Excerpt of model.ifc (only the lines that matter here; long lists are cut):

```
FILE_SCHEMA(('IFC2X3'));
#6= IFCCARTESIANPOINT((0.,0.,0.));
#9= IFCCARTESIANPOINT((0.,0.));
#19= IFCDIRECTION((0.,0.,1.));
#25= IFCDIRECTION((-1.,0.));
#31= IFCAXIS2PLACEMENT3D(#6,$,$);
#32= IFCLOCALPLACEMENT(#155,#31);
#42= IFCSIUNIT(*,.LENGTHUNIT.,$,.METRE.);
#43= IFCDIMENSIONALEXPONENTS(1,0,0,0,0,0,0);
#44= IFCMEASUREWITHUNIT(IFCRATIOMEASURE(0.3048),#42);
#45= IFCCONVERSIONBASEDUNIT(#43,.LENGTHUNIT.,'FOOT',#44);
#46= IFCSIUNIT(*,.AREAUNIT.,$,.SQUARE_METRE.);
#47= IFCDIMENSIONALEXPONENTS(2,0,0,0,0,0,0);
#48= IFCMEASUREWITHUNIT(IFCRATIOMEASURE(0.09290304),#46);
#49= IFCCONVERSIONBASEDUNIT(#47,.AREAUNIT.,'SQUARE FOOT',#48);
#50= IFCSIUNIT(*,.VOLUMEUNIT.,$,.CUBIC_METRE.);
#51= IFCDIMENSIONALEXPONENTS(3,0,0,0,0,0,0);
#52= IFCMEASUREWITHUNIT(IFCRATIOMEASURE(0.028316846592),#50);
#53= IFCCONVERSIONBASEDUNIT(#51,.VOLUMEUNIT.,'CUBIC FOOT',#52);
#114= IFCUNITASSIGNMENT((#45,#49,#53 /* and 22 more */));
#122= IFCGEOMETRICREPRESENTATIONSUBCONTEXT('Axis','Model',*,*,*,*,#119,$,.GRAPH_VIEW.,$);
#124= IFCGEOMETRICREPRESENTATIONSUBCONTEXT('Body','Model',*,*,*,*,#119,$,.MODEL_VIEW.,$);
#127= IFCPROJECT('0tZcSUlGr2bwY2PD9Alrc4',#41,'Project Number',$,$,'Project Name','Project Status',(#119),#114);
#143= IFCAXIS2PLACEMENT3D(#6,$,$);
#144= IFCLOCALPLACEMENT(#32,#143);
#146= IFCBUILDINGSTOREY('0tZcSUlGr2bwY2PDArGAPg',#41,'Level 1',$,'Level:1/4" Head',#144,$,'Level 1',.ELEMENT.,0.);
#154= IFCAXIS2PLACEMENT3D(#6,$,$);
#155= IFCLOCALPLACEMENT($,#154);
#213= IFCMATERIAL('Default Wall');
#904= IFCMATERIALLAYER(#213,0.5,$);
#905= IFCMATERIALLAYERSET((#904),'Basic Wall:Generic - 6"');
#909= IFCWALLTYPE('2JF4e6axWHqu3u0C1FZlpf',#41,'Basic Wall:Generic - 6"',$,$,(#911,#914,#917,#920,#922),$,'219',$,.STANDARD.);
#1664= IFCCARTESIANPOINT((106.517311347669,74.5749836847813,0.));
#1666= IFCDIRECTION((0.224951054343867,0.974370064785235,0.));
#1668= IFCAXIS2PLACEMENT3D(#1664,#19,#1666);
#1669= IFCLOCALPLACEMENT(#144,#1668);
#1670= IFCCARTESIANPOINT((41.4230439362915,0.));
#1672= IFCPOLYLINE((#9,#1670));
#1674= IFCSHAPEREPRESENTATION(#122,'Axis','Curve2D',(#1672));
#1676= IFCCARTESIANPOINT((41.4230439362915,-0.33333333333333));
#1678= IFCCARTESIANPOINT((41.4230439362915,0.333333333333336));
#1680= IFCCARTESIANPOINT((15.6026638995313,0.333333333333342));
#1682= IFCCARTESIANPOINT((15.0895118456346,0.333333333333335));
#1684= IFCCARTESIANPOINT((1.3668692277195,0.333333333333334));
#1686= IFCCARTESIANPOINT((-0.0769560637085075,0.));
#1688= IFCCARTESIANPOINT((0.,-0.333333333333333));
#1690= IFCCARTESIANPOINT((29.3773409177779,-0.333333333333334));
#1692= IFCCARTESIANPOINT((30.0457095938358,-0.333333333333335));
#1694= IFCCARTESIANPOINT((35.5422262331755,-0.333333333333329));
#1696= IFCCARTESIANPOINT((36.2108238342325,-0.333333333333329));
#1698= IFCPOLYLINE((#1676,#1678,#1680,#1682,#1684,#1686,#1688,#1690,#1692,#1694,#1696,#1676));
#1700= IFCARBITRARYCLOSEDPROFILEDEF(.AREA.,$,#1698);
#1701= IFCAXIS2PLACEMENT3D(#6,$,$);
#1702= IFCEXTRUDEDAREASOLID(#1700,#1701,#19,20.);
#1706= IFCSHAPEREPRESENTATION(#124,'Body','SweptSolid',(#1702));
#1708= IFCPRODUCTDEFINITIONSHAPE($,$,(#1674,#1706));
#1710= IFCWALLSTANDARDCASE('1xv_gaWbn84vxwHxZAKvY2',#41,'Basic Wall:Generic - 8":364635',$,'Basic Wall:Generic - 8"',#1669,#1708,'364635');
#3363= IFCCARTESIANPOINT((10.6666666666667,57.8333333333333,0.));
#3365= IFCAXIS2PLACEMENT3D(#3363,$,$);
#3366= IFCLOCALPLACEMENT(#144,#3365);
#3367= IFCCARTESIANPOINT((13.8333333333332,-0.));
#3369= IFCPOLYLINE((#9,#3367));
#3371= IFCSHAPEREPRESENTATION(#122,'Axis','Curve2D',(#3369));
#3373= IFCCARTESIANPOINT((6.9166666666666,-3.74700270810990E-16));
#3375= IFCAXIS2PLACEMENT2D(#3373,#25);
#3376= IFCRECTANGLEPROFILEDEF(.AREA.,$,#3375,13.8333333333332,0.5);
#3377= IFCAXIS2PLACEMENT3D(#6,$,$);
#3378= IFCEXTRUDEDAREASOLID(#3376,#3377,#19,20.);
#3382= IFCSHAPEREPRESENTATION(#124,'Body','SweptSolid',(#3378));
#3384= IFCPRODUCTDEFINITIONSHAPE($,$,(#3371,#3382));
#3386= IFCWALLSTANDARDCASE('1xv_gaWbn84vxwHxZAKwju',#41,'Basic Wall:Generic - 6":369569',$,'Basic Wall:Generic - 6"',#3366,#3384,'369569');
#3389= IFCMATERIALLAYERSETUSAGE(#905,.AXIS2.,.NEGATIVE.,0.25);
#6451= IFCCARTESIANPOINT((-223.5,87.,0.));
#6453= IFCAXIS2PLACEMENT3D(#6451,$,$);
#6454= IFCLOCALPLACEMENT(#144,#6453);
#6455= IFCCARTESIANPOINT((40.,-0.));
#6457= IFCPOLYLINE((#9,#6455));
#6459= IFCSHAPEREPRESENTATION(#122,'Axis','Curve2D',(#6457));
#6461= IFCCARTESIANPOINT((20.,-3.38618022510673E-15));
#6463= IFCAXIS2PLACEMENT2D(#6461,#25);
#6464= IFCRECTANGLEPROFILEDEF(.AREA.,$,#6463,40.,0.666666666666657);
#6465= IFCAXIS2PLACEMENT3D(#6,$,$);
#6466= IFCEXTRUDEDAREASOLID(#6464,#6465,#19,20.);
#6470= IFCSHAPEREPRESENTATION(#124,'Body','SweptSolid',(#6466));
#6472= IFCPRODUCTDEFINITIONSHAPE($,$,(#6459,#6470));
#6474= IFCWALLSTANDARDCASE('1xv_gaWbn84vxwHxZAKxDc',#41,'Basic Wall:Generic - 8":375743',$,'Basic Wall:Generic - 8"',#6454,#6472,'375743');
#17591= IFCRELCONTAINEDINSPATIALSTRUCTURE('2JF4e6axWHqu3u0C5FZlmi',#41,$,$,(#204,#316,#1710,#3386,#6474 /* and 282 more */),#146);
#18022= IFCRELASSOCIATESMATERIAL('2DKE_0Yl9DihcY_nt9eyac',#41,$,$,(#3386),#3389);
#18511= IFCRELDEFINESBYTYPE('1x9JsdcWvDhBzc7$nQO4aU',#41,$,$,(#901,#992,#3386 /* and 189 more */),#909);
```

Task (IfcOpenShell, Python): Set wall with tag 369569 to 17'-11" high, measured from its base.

```python
import ifcopenshell
import ifcopenshell.geom
import ifcopenshell.util.representation
import ifcopenshell.util.shape
import ifcopenshell.util.unit

model = ifcopenshell.open("model.ifc")
unit_scale = ifcopenshell.util.unit.calculate_unit_scale(model)
settings = ifcopenshell.geom.settings()


def volume(element):
    """Net volume in cubic metres, openings subtracted."""
    shape = ifcopenshell.geom.create_shape(settings, element)
    return ifcopenshell.util.shape.get_volume(shape.geometry)


wall = model.by_guid("1xv_gaWbn84vxwHxZAKwju")
before = volume(wall)

body = ifcopenshell.util.representation.get_representation(wall, "Model", "Body")
solid = body.Items[0]
old_height = solid.Depth
solid.Depth = 215 * 0.0254 / unit_scale
after = volume(wall)

print(f"height {old_height:g} -> {solid.Depth:g}, volume {before:.3f} -> {after:.3f} m3")

model.write("model-out.ifc")
```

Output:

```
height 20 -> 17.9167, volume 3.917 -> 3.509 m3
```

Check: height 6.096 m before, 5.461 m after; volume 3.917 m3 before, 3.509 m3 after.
